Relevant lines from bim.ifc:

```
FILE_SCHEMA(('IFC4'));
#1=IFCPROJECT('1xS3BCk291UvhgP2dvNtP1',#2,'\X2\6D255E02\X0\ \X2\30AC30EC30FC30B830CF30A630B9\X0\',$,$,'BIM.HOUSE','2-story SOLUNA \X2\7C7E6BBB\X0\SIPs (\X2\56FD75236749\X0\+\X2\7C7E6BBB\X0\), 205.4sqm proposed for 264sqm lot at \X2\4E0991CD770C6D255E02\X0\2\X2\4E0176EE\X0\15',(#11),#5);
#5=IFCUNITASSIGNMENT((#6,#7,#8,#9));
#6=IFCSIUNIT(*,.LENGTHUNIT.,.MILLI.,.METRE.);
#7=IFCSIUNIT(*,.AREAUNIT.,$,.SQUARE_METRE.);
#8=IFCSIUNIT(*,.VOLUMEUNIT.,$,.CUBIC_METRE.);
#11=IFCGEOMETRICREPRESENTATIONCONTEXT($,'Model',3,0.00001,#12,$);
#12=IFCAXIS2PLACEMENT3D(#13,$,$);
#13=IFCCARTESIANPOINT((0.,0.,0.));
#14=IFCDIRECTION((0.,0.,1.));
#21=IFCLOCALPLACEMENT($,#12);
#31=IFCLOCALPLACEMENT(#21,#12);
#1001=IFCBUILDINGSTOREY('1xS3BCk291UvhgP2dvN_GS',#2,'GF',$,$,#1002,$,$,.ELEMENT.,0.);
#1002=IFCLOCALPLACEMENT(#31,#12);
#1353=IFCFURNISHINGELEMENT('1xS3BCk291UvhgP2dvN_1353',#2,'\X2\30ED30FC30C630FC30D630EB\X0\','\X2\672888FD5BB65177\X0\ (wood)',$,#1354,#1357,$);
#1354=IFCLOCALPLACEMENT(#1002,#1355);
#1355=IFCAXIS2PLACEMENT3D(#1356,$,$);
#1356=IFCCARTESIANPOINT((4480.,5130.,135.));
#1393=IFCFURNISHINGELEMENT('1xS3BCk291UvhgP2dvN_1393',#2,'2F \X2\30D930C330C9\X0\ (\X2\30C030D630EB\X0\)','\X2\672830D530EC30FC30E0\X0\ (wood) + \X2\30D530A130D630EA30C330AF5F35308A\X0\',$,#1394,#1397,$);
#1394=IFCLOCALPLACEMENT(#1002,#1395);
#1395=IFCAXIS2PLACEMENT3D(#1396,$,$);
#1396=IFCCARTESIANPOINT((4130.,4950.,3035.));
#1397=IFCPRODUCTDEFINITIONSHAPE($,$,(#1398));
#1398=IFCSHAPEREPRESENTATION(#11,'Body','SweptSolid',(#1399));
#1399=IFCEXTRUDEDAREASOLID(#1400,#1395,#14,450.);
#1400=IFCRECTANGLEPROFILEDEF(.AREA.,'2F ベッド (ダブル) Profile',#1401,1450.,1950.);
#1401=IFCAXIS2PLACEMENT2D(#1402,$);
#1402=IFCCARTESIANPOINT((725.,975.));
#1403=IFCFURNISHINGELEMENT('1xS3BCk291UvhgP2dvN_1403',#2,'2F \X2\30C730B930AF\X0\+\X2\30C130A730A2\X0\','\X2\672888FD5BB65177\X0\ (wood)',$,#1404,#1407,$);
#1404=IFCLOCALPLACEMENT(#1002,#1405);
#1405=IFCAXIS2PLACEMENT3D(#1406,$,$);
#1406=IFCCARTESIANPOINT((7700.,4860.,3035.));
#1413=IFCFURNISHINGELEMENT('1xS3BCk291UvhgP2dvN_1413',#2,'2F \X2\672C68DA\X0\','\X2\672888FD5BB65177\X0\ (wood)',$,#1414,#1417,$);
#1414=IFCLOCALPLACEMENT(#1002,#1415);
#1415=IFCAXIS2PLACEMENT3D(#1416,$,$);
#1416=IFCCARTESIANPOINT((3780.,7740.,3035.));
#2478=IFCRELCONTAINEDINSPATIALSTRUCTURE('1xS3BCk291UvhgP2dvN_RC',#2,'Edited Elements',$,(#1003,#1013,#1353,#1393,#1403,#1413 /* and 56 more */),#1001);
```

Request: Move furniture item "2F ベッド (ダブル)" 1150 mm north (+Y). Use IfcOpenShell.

```python
import ifcopenshell
import ifcopenshell.api.geometry
import ifcopenshell.util.placement
import ifcopenshell.util.unit

model = ifcopenshell.open("bim.ifc")
unit_scale = ifcopenshell.util.unit.calculate_unit_scale(model)

item = model.by_guid("1xS3BCk291UvhgP2dvN_1393")
matrix = ifcopenshell.util.placement.get_local_placement(item.ObjectPlacement)
matrix[1, 3] += 1.15 / unit_scale
ifcopenshell.api.geometry.edit_object_placement(model, product=item, matrix=matrix, is_si=False)

print(ifcopenshell.util.placement.get_local_placement(item.ObjectPlacement).round(3) + 0.0)

model.write("bim_rev.ifc")
```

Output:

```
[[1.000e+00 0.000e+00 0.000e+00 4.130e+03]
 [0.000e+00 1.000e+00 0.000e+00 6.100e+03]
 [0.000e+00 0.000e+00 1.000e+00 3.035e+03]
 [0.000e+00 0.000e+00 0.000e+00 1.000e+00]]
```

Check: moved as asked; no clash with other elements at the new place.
